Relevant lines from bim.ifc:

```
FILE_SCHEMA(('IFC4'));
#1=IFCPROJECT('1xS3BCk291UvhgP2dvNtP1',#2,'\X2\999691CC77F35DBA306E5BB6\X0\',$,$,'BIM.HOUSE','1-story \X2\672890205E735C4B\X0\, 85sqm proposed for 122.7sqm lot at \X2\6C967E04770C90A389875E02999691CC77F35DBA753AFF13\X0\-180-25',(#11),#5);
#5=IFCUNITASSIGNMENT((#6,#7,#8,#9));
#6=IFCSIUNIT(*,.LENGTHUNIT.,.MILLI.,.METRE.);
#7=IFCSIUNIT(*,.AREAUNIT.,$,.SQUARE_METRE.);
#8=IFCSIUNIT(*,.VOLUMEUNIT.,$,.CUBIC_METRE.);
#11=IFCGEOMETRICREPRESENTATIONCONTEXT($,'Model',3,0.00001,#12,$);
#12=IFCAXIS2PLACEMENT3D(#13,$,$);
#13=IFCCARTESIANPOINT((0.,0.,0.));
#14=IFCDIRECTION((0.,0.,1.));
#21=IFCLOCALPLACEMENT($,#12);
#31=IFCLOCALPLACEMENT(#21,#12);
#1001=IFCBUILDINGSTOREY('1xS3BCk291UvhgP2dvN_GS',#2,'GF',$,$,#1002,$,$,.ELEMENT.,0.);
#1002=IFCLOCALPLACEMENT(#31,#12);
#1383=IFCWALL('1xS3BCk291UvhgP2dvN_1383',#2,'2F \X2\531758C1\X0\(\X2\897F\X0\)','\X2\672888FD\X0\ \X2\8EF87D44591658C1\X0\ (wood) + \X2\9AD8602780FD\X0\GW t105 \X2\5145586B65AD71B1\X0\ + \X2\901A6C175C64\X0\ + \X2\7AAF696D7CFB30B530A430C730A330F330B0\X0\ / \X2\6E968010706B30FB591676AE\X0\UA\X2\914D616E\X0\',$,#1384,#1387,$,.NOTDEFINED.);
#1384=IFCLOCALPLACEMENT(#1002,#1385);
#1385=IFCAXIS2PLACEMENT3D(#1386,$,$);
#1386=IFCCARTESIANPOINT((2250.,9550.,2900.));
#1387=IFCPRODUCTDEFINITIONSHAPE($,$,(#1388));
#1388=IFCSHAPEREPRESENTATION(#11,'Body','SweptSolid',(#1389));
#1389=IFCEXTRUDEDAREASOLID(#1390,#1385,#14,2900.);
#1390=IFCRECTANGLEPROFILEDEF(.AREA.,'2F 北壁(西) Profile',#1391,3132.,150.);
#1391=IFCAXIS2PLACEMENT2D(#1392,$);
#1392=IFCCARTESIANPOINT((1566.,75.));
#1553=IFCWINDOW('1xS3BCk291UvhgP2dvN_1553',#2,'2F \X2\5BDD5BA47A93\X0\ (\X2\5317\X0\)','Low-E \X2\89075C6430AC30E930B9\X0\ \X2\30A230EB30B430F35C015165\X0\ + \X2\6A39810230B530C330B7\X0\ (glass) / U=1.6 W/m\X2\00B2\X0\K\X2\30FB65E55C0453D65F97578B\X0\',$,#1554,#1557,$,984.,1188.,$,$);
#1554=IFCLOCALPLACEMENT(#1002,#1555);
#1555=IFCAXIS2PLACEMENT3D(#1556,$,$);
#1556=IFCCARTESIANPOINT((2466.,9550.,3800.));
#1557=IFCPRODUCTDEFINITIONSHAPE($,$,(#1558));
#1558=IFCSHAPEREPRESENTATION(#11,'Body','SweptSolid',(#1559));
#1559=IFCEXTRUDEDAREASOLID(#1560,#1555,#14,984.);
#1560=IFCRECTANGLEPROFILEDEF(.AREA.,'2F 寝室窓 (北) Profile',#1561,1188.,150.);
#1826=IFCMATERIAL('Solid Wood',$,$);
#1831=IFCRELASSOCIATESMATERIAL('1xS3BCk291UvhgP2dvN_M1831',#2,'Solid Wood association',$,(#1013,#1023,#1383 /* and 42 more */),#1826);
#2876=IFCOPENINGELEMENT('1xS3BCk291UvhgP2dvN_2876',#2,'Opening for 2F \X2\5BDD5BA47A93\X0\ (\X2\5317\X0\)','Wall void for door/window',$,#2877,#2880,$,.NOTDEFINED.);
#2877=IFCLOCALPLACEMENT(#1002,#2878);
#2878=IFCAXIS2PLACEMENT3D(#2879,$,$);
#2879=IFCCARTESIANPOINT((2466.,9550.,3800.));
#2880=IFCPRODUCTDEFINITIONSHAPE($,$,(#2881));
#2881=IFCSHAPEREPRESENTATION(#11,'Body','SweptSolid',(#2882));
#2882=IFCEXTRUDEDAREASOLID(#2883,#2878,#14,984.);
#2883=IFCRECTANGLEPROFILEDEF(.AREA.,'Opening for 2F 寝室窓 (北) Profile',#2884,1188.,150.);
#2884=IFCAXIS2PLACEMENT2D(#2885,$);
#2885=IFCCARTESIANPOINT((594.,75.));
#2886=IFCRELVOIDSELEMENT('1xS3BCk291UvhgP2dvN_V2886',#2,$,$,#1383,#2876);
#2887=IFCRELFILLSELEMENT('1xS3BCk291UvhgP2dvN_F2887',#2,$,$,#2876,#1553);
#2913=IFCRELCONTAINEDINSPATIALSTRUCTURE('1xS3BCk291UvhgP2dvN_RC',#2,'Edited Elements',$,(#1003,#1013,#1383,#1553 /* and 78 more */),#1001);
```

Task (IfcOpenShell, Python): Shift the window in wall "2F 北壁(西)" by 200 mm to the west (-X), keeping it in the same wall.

```python
import ifcopenshell
import ifcopenshell.api.geometry
import ifcopenshell.util.placement
import ifcopenshell.util.unit

model = ifcopenshell.open("bim.ifc")
unit_scale = ifcopenshell.util.unit.calculate_unit_scale(model)

window = model.by_id(1553)
opening = window.FillsVoids[0].RelatingOpeningElement
wall = opening.VoidsElements[0].RelatingBuildingElement

wall_matrix = ifcopenshell.util.placement.get_local_placement(wall.ObjectPlacement)
shift = wall_matrix[:3, 0] * -0.2 / unit_scale
before = ifcopenshell.util.placement.get_local_placement(window.ObjectPlacement)[:3, 3].copy()

# The window is not placed relative to its opening, so move both.
for product in (opening, window):
    matrix = ifcopenshell.util.placement.get_local_placement(product.ObjectPlacement)
    matrix[:3, 3] += shift
    ifcopenshell.api.geometry.edit_object_placement(model, product=product, matrix=matrix, is_si=False)

after = ifcopenshell.util.placement.get_local_placement(window.ObjectPlacement)[:3, 3]
print("window moved by", (after - before).round(3) + 0.0)

model.write("bim_v2.ifc")
```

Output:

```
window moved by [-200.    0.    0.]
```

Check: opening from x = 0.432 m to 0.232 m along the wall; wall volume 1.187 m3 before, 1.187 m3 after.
